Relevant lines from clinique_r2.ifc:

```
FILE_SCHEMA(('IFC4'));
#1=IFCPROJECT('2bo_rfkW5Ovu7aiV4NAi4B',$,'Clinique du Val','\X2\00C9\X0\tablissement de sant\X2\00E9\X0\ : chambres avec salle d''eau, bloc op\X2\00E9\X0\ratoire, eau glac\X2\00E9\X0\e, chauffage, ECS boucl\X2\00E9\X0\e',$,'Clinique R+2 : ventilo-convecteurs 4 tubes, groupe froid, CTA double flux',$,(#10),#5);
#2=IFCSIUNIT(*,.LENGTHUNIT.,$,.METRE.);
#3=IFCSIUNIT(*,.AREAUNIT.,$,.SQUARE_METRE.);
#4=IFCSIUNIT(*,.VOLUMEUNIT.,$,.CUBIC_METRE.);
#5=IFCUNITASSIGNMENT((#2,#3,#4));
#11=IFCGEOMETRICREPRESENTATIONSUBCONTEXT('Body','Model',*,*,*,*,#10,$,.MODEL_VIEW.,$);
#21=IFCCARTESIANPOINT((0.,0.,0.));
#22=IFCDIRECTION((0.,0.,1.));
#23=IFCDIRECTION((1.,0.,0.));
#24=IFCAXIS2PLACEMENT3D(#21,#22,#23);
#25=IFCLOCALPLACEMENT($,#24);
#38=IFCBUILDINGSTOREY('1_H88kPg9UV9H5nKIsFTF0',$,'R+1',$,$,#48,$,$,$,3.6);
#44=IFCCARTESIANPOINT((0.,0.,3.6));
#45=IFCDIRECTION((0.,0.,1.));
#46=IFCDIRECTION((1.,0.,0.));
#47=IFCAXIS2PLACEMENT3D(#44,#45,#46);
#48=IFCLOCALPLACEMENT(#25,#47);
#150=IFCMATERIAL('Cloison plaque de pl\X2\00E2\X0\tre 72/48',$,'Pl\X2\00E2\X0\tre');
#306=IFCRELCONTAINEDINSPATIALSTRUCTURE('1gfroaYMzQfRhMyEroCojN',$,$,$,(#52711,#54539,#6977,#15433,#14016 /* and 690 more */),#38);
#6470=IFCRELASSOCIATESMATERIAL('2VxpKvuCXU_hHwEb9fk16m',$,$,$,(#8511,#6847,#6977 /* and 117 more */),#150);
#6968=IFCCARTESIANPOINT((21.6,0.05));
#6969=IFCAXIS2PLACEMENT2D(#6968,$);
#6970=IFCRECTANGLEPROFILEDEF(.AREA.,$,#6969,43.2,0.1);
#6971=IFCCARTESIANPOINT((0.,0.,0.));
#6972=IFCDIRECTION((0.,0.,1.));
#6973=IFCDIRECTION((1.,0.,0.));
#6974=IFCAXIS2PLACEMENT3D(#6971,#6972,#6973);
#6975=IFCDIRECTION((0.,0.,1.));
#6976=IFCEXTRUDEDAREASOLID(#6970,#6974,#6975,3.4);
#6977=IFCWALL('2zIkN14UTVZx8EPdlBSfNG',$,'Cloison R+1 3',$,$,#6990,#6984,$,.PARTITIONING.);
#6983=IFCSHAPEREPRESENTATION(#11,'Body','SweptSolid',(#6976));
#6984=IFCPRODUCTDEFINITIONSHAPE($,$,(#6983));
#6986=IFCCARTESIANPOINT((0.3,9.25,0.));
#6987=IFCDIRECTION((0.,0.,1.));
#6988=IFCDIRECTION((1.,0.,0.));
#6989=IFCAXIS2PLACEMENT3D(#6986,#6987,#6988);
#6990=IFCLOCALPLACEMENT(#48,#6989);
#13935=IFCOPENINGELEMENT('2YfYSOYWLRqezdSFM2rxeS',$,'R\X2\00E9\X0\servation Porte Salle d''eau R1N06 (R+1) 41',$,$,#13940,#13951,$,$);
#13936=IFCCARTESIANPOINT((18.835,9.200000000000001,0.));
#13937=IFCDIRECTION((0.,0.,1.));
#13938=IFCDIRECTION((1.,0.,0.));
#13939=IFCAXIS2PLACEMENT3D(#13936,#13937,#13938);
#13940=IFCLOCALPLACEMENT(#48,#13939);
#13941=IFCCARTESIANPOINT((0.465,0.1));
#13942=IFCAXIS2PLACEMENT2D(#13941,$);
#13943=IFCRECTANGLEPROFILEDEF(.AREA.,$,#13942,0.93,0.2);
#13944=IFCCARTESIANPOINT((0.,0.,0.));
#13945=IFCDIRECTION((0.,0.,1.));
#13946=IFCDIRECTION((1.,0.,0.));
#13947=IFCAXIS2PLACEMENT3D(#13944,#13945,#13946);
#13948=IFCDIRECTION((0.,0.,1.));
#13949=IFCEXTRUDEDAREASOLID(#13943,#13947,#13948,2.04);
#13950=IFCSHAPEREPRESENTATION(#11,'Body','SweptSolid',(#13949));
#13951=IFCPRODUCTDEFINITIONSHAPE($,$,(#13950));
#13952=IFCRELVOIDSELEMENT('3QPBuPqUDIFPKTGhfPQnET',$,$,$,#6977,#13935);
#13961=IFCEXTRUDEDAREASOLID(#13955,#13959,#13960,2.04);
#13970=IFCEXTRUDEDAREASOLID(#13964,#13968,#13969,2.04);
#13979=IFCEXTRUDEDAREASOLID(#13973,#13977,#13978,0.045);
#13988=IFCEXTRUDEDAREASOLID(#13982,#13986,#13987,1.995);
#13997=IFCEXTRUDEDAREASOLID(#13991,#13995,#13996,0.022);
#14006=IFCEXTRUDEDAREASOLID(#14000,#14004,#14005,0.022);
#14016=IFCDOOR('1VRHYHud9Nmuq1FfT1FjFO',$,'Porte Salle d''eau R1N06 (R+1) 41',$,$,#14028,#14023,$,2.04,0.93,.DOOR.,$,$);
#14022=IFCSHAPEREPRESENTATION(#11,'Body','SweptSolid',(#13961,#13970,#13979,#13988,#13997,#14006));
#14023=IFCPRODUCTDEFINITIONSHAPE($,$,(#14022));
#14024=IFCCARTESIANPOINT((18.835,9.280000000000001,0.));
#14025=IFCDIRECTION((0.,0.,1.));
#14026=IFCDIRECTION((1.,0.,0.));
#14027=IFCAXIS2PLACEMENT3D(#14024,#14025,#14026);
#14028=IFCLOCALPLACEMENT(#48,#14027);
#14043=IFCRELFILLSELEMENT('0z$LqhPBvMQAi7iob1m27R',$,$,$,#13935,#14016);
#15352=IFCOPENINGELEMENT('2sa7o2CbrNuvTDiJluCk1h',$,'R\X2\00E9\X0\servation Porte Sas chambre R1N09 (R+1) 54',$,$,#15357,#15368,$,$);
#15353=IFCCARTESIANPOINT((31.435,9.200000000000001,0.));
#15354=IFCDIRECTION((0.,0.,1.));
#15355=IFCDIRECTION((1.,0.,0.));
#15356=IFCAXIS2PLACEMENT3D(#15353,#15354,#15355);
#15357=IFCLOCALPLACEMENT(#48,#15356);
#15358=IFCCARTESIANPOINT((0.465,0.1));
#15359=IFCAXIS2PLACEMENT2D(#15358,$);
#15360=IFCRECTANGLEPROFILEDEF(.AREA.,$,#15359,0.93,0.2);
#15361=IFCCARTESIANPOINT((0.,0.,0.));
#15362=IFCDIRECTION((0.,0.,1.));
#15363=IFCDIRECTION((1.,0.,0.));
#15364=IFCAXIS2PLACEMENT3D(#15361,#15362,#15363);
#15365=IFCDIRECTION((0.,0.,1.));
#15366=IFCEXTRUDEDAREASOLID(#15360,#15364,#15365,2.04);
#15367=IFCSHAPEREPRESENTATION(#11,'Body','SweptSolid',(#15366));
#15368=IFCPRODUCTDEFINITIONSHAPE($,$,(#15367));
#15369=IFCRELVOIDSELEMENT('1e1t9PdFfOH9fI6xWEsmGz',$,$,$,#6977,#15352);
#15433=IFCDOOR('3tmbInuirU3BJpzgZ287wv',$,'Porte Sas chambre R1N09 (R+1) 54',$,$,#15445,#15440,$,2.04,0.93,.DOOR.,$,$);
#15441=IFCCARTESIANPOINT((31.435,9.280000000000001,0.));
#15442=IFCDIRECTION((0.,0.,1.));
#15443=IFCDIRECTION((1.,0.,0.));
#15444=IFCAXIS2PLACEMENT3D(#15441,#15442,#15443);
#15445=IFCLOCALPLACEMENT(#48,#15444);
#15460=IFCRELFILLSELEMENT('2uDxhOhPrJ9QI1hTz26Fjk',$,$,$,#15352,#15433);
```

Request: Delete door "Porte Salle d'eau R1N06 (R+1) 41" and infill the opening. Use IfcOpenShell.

```python
import ifcopenshell
import ifcopenshell.api.feature
import ifcopenshell.api.root
import ifcopenshell.geom
import ifcopenshell.util.shape

model = ifcopenshell.open("clinique_r2.ifc")
settings = ifcopenshell.geom.settings()


def volume(element):
    """Net volume in cubic metres, openings subtracted."""
    shape = ifcopenshell.geom.create_shape(settings, element)
    return ifcopenshell.util.shape.get_volume(shape.geometry)


door = model.by_guid("1VRHYHud9Nmuq1FfT1FjFO")
opening = door.FillsVoids[0].RelatingOpeningElement
wall = opening.VoidsElements[0].RelatingBuildingElement
before = volume(wall)

ifcopenshell.api.root.remove_product(model, product=door)
ifcopenshell.api.feature.remove_feature(model, feature=opening)

after = volume(wall)

print(f"wall volume {before:.3f} -> {after:.3f} m3")

model.write("clinique_r2_edited.ifc")
```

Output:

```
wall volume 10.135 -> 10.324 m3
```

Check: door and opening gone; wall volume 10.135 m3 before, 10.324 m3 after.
